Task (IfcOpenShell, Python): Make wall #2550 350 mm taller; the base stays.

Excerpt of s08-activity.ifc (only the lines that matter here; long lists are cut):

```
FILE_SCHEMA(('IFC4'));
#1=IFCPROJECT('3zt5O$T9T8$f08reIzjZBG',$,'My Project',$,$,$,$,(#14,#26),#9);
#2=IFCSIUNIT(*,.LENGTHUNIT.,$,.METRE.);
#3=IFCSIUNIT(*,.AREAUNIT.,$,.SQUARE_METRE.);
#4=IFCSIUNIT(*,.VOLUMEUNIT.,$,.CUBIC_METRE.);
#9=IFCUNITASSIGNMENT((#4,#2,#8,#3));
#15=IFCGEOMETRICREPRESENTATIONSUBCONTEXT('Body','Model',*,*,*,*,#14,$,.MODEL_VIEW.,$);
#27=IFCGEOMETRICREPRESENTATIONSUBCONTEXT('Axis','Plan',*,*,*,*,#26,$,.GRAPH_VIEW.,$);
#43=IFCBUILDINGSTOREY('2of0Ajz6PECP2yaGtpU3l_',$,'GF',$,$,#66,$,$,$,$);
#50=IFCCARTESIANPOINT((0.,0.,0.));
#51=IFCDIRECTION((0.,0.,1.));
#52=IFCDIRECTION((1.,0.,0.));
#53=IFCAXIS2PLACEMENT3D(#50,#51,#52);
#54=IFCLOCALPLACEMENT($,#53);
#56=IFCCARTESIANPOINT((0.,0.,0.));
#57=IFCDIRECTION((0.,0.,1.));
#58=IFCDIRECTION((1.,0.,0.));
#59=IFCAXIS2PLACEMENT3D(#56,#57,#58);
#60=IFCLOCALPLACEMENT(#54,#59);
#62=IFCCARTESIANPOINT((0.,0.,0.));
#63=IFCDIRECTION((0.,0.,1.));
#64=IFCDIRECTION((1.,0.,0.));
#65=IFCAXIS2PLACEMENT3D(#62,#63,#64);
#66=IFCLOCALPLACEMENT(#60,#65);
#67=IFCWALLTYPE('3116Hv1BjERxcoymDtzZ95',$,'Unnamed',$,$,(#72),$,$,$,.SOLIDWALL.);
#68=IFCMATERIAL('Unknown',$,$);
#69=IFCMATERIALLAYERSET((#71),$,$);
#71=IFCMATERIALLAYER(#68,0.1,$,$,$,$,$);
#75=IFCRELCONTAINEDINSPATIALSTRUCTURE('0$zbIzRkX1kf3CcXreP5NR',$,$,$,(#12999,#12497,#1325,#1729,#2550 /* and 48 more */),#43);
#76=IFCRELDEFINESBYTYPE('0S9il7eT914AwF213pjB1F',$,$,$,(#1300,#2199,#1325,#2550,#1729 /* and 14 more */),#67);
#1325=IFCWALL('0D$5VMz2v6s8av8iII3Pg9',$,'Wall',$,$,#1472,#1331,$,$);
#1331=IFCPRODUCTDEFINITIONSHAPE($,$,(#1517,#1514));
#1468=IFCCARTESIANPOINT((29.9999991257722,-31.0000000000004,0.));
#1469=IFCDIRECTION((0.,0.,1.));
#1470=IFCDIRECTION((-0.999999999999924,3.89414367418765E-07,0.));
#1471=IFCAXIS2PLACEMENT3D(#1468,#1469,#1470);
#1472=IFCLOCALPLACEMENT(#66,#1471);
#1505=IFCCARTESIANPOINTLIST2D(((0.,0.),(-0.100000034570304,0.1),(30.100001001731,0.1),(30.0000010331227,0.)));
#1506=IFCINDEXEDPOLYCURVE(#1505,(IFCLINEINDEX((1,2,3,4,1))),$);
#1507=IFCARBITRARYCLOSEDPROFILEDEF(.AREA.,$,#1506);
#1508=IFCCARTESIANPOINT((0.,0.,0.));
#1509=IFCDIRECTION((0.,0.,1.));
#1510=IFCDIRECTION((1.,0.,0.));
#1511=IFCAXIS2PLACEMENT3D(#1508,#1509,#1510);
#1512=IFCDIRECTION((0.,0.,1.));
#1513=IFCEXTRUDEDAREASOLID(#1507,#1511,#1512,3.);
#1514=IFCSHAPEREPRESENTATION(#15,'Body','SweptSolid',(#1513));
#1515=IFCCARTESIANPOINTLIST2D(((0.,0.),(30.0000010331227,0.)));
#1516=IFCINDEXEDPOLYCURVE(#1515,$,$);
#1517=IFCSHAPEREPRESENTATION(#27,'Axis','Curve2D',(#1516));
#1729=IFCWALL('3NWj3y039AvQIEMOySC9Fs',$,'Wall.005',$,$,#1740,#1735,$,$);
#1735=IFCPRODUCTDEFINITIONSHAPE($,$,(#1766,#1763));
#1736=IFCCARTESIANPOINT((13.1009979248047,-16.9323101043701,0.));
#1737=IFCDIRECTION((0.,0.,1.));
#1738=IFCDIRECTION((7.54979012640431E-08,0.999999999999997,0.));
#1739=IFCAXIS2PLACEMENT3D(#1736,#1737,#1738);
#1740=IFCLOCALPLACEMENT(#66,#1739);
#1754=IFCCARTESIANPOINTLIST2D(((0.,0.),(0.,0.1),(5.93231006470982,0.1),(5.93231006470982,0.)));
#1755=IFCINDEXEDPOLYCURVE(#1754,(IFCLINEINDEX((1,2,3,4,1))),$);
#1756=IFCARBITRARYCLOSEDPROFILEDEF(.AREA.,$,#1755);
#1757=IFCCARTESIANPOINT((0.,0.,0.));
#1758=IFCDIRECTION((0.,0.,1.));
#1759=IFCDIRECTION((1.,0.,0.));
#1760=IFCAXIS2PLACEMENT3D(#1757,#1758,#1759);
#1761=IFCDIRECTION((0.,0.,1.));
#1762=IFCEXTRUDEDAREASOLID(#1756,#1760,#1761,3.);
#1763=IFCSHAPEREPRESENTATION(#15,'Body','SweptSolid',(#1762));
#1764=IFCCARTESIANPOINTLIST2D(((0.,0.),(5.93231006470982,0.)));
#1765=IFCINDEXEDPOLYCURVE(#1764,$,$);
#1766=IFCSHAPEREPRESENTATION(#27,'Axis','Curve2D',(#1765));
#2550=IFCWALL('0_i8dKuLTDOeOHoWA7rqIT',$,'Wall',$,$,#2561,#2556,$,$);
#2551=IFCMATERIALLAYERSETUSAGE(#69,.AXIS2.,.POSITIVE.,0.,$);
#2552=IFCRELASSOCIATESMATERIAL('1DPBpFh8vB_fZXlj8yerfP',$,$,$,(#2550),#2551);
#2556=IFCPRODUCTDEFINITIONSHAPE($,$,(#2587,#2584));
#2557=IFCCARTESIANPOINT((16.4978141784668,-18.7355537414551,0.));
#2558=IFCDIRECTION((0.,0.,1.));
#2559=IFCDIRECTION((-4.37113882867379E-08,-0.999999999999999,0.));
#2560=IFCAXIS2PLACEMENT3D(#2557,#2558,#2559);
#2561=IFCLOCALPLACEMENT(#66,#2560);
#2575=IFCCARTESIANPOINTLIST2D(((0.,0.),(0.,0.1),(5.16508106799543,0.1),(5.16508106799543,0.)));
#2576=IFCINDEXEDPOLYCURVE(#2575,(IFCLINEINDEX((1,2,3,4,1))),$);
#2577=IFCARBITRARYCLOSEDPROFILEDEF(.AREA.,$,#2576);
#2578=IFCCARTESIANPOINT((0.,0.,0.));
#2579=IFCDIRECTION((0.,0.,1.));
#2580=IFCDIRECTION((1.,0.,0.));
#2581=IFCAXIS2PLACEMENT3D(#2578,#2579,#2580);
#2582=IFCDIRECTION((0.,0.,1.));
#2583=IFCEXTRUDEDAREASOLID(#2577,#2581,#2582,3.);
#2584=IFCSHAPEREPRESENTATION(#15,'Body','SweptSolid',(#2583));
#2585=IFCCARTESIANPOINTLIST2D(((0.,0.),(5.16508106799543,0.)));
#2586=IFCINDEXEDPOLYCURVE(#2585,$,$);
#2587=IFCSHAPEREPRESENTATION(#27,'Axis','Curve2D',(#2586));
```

```python
import ifcopenshell
import ifcopenshell.geom
import ifcopenshell.util.representation
import ifcopenshell.util.shape
import ifcopenshell.util.unit

model = ifcopenshell.open("s08-activity.ifc")
unit_scale = ifcopenshell.util.unit.calculate_unit_scale(model)
settings = ifcopenshell.geom.settings()


def volume(element):
    """Net volume in cubic metres, openings subtracted."""
    shape = ifcopenshell.geom.create_shape(settings, element)
    return ifcopenshell.util.shape.get_volume(shape.geometry)


wall = model.by_guid("0_i8dKuLTDOeOHoWA7rqIT")
before = volume(wall)

body = ifcopenshell.util.representation.get_representation(wall, "Model", "Body")
solid = body.Items[0]
old_height = solid.Depth
solid.Depth += 0.35 / unit_scale
after = volume(wall)

print(f"height {old_height:g} -> {solid.Depth:g}, volume {before:.3f} -> {after:.3f} m3")

model.write("s08-activity_v2.ifc")
```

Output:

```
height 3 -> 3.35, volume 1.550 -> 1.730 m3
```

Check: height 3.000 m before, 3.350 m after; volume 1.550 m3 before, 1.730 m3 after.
